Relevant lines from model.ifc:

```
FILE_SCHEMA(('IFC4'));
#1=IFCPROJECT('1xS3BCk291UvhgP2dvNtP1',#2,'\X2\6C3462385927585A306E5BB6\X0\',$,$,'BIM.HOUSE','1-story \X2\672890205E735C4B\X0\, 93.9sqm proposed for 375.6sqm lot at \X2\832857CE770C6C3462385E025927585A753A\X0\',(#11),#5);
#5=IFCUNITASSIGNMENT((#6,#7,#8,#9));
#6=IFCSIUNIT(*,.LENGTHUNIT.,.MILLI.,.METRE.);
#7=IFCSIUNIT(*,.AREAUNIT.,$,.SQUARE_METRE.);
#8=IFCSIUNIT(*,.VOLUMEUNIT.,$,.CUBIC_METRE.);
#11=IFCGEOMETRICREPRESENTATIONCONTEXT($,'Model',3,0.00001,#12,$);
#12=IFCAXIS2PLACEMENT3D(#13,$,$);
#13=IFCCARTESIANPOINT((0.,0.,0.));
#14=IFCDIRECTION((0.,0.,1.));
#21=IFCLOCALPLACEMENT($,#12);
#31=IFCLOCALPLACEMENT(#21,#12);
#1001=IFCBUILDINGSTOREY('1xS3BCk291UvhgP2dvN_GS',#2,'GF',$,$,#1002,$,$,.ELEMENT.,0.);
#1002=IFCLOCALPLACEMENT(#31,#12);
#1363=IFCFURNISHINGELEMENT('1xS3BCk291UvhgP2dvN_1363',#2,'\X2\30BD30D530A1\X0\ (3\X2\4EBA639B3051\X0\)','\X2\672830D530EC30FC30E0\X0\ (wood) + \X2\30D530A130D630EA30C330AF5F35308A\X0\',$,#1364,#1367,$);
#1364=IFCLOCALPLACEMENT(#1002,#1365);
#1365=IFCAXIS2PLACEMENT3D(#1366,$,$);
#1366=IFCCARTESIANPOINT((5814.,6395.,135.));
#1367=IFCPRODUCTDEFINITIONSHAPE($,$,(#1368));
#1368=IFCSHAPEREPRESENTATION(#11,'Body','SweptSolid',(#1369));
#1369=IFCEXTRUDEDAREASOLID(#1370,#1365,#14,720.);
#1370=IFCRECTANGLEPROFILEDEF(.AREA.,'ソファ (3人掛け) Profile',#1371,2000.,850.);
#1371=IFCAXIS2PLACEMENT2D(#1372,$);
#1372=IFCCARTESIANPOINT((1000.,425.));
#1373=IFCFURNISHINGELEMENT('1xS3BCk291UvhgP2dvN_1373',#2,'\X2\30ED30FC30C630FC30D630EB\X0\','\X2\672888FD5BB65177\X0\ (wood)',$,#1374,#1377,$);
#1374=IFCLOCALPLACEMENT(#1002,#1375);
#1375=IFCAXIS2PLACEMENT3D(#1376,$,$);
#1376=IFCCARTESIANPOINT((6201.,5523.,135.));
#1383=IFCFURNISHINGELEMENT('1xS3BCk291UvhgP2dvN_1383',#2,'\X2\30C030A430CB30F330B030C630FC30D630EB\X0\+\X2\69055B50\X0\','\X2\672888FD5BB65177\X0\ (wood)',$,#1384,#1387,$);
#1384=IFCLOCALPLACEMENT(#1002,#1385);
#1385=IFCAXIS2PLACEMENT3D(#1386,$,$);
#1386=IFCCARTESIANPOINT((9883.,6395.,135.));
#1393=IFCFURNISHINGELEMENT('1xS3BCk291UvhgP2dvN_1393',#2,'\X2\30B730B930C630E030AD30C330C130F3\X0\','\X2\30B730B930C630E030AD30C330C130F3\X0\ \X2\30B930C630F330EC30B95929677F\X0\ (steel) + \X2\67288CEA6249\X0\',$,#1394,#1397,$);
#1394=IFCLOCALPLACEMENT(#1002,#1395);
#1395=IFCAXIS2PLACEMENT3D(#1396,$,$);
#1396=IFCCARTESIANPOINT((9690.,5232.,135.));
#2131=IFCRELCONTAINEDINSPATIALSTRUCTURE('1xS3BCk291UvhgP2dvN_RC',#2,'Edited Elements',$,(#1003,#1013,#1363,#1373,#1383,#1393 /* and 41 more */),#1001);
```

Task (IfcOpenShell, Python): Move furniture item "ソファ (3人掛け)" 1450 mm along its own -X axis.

```python
import ifcopenshell
import ifcopenshell.api.geometry
import ifcopenshell.util.placement
import ifcopenshell.util.unit

model = ifcopenshell.open("model.ifc")
unit_scale = ifcopenshell.util.unit.calculate_unit_scale(model)

item = model.by_guid("1xS3BCk291UvhgP2dvN_1363")
matrix = ifcopenshell.util.placement.get_local_placement(item.ObjectPlacement)
matrix[:3, 3] -= matrix[:3, 0] * 1.45 / unit_scale
ifcopenshell.api.geometry.edit_object_placement(model, product=item, matrix=matrix, is_si=False)

print(ifcopenshell.util.placement.get_local_placement(item.ObjectPlacement).round(3) + 0.0)

model.write("model_v2.ifc")
```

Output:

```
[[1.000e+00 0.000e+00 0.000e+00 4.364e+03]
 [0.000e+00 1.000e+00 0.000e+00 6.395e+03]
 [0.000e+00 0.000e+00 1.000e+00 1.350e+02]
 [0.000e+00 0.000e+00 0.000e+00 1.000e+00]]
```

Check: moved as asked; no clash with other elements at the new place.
